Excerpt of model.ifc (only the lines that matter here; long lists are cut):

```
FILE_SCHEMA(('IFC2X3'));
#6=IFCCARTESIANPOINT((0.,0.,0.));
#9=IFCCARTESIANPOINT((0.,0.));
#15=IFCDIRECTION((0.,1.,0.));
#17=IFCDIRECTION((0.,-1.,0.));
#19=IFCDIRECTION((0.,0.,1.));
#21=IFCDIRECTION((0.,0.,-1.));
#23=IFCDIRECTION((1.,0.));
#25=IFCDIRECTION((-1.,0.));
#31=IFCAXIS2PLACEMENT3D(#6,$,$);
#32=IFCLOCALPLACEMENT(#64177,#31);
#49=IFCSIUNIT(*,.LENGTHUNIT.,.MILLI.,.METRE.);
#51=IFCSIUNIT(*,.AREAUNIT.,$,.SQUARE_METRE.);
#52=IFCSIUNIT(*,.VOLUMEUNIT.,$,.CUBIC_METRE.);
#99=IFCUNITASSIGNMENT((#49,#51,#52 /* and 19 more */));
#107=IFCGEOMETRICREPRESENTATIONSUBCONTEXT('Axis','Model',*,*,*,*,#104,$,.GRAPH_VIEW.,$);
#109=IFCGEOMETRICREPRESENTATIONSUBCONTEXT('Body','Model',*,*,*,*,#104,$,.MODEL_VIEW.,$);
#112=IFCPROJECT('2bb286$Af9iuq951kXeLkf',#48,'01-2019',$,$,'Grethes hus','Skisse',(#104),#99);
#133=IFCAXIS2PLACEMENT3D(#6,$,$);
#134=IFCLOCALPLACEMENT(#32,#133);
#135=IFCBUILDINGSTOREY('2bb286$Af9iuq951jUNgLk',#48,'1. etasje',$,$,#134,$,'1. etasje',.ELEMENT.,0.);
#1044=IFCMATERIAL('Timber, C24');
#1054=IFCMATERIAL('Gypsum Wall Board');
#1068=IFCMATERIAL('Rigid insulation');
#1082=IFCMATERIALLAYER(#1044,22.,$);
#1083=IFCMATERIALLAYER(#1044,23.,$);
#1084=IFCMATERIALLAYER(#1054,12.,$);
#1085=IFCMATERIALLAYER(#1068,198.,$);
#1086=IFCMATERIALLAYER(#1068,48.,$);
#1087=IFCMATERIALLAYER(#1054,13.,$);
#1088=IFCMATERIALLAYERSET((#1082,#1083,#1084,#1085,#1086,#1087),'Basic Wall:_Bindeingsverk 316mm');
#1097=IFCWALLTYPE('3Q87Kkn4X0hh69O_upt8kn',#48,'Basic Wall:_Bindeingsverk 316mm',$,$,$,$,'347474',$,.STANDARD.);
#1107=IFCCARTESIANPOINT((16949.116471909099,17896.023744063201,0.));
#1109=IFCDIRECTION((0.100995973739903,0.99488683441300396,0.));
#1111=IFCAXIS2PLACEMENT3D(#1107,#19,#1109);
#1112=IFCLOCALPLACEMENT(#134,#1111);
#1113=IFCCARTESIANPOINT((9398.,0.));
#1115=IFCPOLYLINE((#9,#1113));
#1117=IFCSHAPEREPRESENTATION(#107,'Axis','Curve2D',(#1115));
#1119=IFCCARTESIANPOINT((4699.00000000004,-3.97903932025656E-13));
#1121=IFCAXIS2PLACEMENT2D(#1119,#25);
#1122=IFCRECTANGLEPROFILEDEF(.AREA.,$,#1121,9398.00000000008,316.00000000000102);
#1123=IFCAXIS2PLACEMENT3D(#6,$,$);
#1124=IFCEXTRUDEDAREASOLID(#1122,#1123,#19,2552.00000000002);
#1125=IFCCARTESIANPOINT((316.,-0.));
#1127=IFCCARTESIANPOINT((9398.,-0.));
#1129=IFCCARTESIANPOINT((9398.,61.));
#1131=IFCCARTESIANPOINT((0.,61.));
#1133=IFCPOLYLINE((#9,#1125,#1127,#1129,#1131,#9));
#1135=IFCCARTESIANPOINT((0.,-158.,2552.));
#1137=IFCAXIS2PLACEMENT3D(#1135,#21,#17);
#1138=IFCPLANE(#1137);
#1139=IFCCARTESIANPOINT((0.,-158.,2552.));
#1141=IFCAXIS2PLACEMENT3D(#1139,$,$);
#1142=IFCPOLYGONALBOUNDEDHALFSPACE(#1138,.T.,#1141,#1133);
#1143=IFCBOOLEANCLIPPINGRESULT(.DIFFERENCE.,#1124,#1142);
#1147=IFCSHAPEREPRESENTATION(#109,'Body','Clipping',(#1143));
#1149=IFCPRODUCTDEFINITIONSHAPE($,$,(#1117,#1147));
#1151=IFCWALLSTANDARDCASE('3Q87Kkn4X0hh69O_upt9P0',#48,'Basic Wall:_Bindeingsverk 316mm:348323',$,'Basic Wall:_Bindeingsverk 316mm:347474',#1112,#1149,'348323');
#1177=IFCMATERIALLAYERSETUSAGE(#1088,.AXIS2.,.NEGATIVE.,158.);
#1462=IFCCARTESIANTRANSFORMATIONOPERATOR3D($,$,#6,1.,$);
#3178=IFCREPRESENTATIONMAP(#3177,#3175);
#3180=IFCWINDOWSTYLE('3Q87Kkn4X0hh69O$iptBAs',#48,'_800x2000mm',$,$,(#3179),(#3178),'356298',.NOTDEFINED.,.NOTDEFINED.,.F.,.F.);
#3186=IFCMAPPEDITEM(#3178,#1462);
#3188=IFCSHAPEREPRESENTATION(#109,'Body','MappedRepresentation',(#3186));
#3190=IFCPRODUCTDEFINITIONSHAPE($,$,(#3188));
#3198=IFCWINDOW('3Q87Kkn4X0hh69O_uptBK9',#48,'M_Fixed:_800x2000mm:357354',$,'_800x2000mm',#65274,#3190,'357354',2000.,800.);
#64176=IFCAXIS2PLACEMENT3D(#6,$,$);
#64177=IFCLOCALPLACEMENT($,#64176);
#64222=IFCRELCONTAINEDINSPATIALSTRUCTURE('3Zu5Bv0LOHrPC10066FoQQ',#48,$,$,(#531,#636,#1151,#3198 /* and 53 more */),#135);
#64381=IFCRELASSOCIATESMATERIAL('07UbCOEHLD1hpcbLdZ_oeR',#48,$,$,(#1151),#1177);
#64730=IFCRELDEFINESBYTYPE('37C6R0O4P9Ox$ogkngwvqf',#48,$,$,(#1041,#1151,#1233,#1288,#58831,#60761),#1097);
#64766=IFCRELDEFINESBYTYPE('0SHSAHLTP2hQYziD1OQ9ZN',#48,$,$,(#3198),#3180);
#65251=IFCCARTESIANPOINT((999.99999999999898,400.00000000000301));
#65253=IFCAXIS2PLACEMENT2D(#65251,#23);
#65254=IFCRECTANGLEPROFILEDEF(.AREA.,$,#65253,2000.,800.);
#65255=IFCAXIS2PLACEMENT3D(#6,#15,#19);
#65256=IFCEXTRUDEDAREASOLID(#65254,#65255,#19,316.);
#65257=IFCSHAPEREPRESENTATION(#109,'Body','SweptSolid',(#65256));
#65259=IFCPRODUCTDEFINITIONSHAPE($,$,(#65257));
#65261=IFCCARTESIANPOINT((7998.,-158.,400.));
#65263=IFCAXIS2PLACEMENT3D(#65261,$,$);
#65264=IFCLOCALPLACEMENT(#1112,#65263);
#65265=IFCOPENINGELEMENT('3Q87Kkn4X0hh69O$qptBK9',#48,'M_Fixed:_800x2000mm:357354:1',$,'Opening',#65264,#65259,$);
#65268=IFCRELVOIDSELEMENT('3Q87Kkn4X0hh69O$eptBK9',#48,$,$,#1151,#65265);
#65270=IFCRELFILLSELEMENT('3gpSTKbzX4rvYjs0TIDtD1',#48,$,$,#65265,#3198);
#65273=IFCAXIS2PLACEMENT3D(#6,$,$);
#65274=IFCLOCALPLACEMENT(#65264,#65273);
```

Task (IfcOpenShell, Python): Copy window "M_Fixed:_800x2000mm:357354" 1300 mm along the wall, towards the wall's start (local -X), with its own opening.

```python
import ifcopenshell
import ifcopenshell.api.feature
import ifcopenshell.api.geometry
import ifcopenshell.api.root
import ifcopenshell.geom
import ifcopenshell.util.element
import ifcopenshell.util.placement
import ifcopenshell.util.shape
import ifcopenshell.util.unit

model = ifcopenshell.open("model.ifc")
unit_scale = ifcopenshell.util.unit.calculate_unit_scale(model)
settings = ifcopenshell.geom.settings()


def volume(element):
    """Net volume in cubic metres, openings subtracted."""
    shape = ifcopenshell.geom.create_shape(settings, element)
    return ifcopenshell.util.shape.get_volume(shape.geometry)


def reuse_history(source, copy):
    """copy_class also copies each property set's owner history, people and application; keep the originals."""
    for rel in copy.IsDefinedBy:
        if rel.is_a("IfcRelDefinesByProperties") and (history := rel.RelatingPropertyDefinition.OwnerHistory):
            rel.RelatingPropertyDefinition.OwnerHistory = source.OwnerHistory
            ifcopenshell.util.element.remove_deep2(model, history)


window = model.by_id(3198)
opening = window.FillsVoids[0].RelatingOpeningElement
wall = opening.VoidsElements[0].RelatingBuildingElement
before = volume(wall)
shift = ifcopenshell.util.placement.get_local_placement(wall.ObjectPlacement)[:3, 0] * -1.3 / unit_scale

# copy_class copies the void relationship, type, container and properties, but no geometry.
new_opening = ifcopenshell.api.root.copy_class(model, product=opening)
new_opening.Representation = ifcopenshell.util.element.copy_deep(
    model, opening.Representation, exclude=["IfcGeometricRepresentationContext", "IfcRepresentationMap"]
)
new_opening.Name = "M_Fixed:_800x2000mm"
new_window = ifcopenshell.api.root.copy_class(model, product=window)
new_window.Representation = ifcopenshell.util.element.copy_deep(
    model, window.Representation, exclude=["IfcGeometricRepresentationContext", "IfcRepresentationMap"]
)
new_window.Name = "M_Fixed:_800x2000mm"
new_window.Tag = None
reuse_history(window, new_window)
fills = ifcopenshell.api.feature.add_filling(model, opening=new_opening, element=new_window)
fills.OwnerHistory = new_window.OwnerHistory  # required in IFC2X3

for old, new in ((opening, new_opening), (window, new_window)):
    matrix = ifcopenshell.util.placement.get_local_placement(old.ObjectPlacement)
    matrix[:3, 3] += shift
    ifcopenshell.api.geometry.edit_object_placement(model, product=new, matrix=matrix, is_si=False)

after = volume(wall)

print(f"wall volume {before:.3f} -> {after:.3f} m3")

model.write("model_v2.ifc")
```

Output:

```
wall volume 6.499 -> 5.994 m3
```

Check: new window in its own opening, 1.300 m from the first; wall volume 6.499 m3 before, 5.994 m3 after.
